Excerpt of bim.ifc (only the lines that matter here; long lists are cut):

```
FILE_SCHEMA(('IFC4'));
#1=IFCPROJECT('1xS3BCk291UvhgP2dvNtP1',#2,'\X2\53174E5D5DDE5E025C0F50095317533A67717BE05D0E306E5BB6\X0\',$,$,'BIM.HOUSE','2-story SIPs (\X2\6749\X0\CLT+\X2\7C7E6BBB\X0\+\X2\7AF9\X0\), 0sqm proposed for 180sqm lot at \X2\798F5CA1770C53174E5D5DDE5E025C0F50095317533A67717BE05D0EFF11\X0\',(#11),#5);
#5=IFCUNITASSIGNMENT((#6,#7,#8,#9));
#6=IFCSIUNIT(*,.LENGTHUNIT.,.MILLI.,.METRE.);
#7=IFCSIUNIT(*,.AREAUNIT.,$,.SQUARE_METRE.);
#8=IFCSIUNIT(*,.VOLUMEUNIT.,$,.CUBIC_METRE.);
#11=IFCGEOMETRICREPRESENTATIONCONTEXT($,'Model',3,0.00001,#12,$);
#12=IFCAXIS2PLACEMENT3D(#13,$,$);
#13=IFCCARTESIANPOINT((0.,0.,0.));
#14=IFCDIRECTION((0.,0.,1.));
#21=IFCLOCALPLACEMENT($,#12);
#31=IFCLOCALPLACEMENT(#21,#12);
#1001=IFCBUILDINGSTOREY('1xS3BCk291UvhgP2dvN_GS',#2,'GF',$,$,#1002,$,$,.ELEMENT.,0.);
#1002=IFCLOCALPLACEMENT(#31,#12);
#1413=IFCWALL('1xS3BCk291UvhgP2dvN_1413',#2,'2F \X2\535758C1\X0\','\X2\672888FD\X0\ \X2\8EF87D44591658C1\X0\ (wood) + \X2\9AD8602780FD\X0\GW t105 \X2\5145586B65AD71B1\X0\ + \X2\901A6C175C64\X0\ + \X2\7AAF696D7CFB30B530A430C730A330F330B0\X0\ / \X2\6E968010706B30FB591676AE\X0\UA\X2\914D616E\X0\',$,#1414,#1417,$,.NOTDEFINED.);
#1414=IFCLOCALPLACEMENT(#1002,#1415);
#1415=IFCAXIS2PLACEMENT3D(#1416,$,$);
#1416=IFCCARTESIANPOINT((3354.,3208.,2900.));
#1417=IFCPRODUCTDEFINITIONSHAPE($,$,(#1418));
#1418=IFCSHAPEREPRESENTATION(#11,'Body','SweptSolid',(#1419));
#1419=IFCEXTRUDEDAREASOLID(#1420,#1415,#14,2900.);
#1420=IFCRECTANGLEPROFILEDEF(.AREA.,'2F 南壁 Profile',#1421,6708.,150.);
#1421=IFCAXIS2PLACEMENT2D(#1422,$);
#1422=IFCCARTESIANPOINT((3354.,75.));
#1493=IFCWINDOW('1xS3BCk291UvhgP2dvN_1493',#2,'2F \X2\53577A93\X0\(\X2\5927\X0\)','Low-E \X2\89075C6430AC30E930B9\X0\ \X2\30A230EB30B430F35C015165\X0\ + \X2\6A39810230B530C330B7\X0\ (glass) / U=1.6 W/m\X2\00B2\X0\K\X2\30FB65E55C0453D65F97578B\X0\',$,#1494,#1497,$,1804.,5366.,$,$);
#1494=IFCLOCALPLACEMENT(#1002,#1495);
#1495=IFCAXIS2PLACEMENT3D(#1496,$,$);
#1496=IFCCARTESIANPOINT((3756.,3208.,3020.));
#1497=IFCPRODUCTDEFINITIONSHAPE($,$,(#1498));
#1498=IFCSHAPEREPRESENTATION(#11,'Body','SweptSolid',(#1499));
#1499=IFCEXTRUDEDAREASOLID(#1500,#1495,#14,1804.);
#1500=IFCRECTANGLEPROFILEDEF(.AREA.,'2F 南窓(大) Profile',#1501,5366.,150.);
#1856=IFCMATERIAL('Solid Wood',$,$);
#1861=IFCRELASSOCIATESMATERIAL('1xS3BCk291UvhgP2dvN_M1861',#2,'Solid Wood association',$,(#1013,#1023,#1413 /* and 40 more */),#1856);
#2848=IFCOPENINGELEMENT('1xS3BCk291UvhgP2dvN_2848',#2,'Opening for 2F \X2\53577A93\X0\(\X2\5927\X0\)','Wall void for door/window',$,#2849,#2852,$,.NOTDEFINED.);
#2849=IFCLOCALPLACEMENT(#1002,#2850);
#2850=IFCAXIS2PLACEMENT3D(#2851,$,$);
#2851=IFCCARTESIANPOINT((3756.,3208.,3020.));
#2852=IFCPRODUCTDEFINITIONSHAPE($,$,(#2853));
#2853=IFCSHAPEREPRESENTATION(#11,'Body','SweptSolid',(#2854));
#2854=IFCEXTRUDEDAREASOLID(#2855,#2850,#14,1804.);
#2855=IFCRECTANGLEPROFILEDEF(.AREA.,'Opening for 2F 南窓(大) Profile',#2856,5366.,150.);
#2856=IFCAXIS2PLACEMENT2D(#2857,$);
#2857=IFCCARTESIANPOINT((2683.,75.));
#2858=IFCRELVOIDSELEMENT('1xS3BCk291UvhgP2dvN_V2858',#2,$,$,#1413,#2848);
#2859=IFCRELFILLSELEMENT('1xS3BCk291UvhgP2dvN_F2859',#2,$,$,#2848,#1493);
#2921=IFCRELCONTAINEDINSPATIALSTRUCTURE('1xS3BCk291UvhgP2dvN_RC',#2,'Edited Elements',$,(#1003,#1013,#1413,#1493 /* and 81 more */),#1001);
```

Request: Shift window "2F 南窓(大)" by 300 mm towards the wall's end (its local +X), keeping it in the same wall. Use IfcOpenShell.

```python
import ifcopenshell
import ifcopenshell.api.geometry
import ifcopenshell.util.placement

model = ifcopenshell.open("bim.ifc")

window = model.by_guid("1xS3BCk291UvhgP2dvN_1493")
opening = window.FillsVoids[0].RelatingOpeningElement
wall = opening.VoidsElements[0].RelatingBuildingElement

wall_matrix = ifcopenshell.util.placement.get_local_placement(wall.ObjectPlacement)
shift = wall_matrix[:3, 0] * 300.0
before = ifcopenshell.util.placement.get_local_placement(window.ObjectPlacement)[:3, 3].copy()

# The window is not placed relative to its opening, so move both.
for product in (opening, window):
    matrix = ifcopenshell.util.placement.get_local_placement(product.ObjectPlacement)
    matrix[:3, 3] += shift
    ifcopenshell.api.geometry.edit_object_placement(model, product=product, matrix=matrix, is_si=False)

after = ifcopenshell.util.placement.get_local_placement(window.ObjectPlacement)[:3, 3]
print("window moved by", (after - before).round(3) + 0.0)

model.write("bim_rev.ifc")
```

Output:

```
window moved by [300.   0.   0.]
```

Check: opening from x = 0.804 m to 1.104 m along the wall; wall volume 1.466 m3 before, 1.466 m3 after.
